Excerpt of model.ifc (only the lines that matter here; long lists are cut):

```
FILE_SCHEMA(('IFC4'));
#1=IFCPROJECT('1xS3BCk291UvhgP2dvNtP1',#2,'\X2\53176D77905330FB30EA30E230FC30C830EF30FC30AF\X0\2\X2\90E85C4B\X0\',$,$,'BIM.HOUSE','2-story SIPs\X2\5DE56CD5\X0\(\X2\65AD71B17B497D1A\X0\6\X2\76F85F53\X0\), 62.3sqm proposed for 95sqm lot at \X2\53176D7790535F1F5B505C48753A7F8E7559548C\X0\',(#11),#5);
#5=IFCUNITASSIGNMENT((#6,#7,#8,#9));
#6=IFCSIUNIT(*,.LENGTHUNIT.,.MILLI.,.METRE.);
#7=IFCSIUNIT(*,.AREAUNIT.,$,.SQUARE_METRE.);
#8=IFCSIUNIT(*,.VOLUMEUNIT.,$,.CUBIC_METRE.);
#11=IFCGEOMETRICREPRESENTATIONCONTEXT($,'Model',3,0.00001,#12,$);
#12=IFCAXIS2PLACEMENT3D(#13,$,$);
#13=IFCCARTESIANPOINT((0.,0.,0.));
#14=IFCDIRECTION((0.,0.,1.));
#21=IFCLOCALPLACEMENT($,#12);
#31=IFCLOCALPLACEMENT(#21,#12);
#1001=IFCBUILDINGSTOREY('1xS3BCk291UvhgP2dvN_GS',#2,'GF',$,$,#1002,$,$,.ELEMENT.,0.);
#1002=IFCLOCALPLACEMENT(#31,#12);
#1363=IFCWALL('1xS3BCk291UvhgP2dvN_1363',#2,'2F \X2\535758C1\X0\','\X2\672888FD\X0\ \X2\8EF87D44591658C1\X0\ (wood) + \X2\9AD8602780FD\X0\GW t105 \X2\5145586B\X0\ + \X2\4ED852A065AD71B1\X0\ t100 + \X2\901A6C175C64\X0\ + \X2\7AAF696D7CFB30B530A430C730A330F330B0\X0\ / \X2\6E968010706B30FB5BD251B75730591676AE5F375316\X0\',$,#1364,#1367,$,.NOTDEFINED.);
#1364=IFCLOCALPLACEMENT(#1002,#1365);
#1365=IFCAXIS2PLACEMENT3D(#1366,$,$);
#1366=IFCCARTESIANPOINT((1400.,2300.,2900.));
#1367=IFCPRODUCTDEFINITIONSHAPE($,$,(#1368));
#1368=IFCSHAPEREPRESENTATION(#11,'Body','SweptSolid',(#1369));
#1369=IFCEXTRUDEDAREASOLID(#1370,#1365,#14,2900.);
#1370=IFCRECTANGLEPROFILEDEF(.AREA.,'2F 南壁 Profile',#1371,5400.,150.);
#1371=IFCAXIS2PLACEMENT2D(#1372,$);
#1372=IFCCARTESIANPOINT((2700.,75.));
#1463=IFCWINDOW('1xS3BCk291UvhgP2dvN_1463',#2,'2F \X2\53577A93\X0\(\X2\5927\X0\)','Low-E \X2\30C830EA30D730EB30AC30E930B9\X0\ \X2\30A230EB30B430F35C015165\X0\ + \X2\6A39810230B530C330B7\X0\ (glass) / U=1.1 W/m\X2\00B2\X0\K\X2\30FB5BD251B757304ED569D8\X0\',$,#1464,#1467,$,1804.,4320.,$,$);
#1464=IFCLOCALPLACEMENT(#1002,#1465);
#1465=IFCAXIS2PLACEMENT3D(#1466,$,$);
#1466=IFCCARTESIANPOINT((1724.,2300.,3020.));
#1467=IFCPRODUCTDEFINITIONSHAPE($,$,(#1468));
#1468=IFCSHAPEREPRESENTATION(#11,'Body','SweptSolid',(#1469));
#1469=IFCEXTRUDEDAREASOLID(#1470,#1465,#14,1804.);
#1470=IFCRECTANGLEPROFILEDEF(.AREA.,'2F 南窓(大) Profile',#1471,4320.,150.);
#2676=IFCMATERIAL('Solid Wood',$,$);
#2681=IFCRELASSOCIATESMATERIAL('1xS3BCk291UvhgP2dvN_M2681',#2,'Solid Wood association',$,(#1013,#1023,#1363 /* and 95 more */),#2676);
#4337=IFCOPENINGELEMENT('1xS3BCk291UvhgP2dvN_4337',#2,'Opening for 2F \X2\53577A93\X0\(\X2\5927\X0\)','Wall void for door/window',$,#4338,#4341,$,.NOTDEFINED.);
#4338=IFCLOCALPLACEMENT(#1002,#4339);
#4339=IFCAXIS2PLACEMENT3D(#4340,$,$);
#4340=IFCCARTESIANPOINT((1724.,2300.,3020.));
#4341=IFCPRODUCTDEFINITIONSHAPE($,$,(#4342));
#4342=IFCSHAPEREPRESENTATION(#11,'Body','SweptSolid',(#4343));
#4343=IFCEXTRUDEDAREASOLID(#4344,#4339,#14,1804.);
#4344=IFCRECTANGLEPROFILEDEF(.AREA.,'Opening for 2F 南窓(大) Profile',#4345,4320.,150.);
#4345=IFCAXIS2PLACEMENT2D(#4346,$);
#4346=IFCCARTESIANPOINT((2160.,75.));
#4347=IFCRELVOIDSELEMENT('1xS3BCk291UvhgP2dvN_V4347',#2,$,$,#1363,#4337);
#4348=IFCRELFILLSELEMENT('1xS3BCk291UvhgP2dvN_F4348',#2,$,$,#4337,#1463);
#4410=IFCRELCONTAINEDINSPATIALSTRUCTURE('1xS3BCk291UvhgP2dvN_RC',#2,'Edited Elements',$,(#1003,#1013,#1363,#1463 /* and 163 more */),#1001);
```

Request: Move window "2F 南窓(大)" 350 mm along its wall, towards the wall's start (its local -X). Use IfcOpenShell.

```python
import ifcopenshell
import ifcopenshell.api.geometry
import ifcopenshell.util.placement

model = ifcopenshell.open("model.ifc")

window = model.by_id(1463)
opening = window.FillsVoids[0].RelatingOpeningElement
wall = opening.VoidsElements[0].RelatingBuildingElement

wall_matrix = ifcopenshell.util.placement.get_local_placement(wall.ObjectPlacement)
shift = wall_matrix[:3, 0] * -350.0
before = ifcopenshell.util.placement.get_local_placement(window.ObjectPlacement)[:3, 3].copy()

# The window is not placed relative to its opening, so move both.
for product in (opening, window):
    matrix = ifcopenshell.util.placement.get_local_placement(product.ObjectPlacement)
    matrix[:3, 3] += shift
    ifcopenshell.api.geometry.edit_object_placement(model, product=product, matrix=matrix, is_si=False)

after = ifcopenshell.util.placement.get_local_placement(window.ObjectPlacement)[:3, 3]
print("window moved by", (after - before).round(3) + 0.0)

model.write("model_v2.ifc")
```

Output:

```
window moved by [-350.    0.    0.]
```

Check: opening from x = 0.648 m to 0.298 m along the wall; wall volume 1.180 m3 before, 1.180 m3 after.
